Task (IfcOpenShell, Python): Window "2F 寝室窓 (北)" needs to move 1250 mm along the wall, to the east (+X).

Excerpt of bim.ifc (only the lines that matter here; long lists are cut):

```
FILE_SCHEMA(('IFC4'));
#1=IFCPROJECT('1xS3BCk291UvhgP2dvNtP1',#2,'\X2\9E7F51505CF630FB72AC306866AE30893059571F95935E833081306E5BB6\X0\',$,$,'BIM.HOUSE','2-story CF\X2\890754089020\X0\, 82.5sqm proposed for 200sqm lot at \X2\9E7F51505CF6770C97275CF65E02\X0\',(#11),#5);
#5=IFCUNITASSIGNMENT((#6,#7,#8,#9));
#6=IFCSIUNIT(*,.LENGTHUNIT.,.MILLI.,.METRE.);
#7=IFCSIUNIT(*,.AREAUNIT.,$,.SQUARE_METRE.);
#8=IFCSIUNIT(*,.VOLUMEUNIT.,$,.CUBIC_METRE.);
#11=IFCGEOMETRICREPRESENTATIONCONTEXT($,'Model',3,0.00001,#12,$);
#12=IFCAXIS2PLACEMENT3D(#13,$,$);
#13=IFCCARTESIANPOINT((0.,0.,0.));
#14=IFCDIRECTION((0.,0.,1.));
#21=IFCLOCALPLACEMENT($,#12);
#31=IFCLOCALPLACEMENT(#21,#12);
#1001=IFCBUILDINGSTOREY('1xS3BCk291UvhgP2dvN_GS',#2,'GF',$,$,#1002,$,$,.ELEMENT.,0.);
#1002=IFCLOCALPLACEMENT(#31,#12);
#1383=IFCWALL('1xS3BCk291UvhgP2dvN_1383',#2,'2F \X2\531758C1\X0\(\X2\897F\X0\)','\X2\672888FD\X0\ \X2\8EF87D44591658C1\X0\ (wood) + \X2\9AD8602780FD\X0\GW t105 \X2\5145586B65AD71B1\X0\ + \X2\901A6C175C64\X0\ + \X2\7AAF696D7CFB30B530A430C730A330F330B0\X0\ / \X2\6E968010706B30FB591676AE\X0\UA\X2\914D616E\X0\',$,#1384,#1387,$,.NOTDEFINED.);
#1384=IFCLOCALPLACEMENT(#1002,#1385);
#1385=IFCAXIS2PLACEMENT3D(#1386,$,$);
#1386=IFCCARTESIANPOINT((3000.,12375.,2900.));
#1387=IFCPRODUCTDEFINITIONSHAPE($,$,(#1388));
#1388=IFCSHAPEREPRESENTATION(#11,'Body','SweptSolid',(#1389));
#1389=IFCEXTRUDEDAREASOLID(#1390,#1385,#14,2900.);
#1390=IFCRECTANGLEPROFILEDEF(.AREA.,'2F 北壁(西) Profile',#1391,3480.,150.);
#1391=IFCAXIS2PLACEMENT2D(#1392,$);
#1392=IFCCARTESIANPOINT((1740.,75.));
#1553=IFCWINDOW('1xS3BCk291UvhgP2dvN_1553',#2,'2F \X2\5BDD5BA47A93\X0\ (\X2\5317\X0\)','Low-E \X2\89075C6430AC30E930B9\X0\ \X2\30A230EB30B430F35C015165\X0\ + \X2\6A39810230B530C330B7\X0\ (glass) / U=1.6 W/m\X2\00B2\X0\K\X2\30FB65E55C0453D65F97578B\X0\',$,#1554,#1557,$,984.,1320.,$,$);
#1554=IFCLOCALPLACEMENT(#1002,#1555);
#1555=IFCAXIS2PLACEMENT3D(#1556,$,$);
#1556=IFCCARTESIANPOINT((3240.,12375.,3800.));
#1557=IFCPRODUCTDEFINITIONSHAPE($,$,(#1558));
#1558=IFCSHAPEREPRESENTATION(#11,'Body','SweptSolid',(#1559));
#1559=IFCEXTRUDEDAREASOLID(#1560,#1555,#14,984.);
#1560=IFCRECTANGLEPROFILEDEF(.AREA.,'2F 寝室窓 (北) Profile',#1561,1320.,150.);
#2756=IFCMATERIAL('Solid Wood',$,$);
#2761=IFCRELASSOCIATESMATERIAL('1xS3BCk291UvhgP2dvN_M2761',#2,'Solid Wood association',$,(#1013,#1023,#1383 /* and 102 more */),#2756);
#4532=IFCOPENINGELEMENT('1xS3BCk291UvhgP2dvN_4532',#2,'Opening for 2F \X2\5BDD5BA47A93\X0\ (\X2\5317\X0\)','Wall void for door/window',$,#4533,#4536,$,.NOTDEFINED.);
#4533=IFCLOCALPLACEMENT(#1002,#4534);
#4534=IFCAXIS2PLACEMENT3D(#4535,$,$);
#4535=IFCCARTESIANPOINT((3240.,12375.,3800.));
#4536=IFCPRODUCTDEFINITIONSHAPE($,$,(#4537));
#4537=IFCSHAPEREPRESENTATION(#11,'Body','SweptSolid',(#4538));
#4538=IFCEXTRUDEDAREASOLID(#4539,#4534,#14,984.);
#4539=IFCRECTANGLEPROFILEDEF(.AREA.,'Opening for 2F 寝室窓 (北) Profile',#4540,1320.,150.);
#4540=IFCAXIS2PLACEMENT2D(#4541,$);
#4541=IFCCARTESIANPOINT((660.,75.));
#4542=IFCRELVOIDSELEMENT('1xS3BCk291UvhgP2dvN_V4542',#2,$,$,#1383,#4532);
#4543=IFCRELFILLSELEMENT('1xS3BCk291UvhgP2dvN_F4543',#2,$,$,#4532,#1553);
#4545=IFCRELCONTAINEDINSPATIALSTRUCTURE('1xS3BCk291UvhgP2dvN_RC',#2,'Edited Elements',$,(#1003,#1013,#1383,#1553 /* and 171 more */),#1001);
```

```python
import ifcopenshell
import ifcopenshell.api.geometry
import ifcopenshell.util.placement

model = ifcopenshell.open("bim.ifc")

window = model.by_guid("1xS3BCk291UvhgP2dvN_1553")
opening = window.FillsVoids[0].RelatingOpeningElement
wall = opening.VoidsElements[0].RelatingBuildingElement

wall_matrix = ifcopenshell.util.placement.get_local_placement(wall.ObjectPlacement)
shift = wall_matrix[:3, 0] * 1250.0
before = ifcopenshell.util.placement.get_local_placement(window.ObjectPlacement)[:3, 3].copy()

# The window is not placed relative to its opening, so move both.
for product in (opening, window):
    matrix = ifcopenshell.util.placement.get_local_placement(product.ObjectPlacement)
    matrix[:3, 3] += shift
    ifcopenshell.api.geometry.edit_object_placement(model, product=product, matrix=matrix, is_si=False)

after = ifcopenshell.util.placement.get_local_placement(window.ObjectPlacement)[:3, 3]
print("window moved by", (after - before).round(3) + 0.0)

model.write("bim_rev.ifc")
```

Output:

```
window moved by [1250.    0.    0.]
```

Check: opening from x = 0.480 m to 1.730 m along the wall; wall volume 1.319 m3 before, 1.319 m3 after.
